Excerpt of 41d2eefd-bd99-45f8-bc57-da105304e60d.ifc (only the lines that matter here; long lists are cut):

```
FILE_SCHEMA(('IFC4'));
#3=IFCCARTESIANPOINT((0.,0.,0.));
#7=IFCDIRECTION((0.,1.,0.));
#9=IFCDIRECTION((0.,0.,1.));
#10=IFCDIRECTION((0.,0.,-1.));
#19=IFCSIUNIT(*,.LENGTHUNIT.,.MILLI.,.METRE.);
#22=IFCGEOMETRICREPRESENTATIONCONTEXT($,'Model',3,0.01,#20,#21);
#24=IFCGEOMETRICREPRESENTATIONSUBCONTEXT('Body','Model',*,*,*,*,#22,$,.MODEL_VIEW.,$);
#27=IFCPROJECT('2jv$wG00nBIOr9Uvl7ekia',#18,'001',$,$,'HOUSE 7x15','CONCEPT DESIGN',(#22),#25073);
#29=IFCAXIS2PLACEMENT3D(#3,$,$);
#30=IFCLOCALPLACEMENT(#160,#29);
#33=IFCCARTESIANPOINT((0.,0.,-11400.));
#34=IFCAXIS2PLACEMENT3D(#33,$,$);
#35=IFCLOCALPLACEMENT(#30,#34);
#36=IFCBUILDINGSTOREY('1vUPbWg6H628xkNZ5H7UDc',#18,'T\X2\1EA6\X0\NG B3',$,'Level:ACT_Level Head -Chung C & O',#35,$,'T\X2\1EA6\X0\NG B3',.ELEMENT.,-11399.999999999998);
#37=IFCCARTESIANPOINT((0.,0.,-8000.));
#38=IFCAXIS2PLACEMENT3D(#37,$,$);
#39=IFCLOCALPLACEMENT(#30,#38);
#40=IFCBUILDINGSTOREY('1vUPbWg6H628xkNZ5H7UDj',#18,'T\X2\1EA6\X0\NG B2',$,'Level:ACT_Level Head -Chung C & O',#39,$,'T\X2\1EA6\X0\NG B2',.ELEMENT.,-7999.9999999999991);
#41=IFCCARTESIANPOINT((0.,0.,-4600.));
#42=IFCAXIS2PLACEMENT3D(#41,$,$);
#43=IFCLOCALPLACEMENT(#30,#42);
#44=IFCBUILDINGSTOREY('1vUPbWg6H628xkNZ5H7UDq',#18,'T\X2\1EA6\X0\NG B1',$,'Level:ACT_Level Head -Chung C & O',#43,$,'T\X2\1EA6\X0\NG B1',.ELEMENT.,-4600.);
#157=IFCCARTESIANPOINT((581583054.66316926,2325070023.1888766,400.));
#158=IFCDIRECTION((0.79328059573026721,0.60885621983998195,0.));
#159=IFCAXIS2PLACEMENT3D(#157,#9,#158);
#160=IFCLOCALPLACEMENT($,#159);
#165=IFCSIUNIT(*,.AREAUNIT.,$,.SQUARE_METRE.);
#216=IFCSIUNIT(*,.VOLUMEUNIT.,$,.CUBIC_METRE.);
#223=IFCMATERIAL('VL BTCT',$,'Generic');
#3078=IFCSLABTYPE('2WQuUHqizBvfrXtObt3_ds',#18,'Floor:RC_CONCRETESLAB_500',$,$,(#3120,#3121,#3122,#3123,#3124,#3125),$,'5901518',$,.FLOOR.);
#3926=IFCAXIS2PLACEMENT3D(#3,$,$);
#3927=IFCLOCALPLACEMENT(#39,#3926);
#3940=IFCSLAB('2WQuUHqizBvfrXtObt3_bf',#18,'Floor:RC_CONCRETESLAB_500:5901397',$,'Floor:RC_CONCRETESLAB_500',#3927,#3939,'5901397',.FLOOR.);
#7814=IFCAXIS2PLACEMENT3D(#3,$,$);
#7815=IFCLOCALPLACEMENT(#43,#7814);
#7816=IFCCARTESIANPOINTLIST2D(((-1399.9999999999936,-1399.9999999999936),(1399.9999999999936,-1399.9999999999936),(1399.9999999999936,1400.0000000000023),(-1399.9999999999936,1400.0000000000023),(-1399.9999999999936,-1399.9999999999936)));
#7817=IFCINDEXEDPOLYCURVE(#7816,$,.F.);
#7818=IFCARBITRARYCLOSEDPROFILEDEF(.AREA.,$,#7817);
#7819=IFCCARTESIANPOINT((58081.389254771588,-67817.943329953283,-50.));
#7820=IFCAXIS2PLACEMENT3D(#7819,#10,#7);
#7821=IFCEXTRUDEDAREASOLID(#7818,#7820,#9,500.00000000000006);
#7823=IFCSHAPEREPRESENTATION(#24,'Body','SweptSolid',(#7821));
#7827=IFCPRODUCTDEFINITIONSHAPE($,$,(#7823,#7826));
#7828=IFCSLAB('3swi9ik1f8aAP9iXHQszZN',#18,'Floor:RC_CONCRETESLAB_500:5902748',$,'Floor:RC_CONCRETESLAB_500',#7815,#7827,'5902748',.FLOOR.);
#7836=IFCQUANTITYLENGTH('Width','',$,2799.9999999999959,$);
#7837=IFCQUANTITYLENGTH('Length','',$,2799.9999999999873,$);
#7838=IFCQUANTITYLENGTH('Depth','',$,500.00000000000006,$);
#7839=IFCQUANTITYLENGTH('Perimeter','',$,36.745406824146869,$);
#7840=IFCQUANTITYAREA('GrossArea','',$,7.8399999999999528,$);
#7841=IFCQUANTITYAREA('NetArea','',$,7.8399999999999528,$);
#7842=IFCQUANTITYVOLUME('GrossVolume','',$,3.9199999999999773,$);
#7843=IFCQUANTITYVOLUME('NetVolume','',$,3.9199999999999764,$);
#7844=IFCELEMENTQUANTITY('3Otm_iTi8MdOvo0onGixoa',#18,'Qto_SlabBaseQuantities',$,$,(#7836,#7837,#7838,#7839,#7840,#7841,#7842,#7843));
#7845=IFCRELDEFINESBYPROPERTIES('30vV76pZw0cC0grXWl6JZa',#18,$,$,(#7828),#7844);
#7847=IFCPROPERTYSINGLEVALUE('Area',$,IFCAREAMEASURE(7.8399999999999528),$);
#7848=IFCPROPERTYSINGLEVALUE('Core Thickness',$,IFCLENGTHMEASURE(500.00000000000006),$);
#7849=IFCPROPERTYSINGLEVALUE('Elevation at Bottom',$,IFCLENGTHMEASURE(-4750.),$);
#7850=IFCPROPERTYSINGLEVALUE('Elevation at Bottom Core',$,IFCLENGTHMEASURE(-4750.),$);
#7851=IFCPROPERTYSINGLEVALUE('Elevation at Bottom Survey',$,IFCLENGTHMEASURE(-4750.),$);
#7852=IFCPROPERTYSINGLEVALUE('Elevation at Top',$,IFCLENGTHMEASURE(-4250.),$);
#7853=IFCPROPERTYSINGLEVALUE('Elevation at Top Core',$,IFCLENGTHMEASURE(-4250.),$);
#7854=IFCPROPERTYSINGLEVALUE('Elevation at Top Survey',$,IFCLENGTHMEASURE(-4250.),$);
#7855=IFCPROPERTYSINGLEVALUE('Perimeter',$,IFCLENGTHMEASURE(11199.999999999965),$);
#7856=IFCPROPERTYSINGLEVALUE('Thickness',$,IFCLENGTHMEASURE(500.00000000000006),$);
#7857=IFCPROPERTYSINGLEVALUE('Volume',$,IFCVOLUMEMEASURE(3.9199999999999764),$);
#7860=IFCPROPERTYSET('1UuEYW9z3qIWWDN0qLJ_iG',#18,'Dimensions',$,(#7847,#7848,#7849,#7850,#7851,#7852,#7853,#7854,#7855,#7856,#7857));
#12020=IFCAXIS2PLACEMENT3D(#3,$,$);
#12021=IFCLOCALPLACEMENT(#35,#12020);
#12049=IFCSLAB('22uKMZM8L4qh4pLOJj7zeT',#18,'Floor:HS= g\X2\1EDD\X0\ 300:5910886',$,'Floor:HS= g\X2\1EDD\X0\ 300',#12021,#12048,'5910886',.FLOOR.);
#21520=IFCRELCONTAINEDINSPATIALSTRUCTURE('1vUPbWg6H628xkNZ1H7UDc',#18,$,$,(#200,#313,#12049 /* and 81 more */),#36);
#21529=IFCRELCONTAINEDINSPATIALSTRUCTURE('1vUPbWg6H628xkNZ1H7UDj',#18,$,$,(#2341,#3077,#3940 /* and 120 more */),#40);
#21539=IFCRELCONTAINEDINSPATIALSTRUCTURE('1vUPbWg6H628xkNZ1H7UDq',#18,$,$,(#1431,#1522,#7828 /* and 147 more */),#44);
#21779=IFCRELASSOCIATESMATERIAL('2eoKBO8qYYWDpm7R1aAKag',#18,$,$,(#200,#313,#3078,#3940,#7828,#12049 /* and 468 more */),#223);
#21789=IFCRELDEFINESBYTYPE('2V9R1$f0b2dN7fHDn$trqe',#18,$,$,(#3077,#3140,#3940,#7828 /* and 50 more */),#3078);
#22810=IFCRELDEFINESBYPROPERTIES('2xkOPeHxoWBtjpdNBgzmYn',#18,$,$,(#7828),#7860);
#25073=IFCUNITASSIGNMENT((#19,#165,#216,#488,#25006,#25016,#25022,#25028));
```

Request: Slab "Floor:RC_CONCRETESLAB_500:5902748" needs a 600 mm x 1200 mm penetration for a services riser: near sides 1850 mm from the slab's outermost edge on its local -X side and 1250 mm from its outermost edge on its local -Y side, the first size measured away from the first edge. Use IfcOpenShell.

```python
import numpy as np
import ifcopenshell
import ifcopenshell.api.feature
import ifcopenshell.api.geometry
import ifcopenshell.api.pset
import ifcopenshell.api.root
import ifcopenshell.geom
import ifcopenshell.util.element
import ifcopenshell.util.placement
import ifcopenshell.util.representation
import ifcopenshell.util.shape
import ifcopenshell.util.unit

model = ifcopenshell.open("41d2eefd-bd99-45f8-bc57-da105304e60d.ifc")
unit_scale = ifcopenshell.util.unit.calculate_unit_scale(model)
area_scale = ifcopenshell.util.unit.calculate_unit_scale(model, "AREAUNIT")
volume_scale = ifcopenshell.util.unit.calculate_unit_scale(model, "VOLUMEUNIT")
settings = ifcopenshell.geom.settings()


def volume(element):
    """Net volume in cubic metres, openings subtracted."""
    shape = ifcopenshell.geom.create_shape(settings, element)
    return ifcopenshell.util.shape.get_volume(shape.geometry)


slab = model.by_guid("3swi9ik1f8aAP9iXHQszZN")
before = volume(slab)

# Extent in the slab's own axes, in metres. The edges named are its -X and -Y sides.
slab_shape = ifcopenshell.geom.create_shape(settings, slab)
vertices = ifcopenshell.util.shape.get_vertices(slab_shape.geometry)
x_min, y_min, bottom = vertices.min(axis=0)
top = vertices[:, 2].max()

opening = ifcopenshell.api.root.create_entity(model, ifc_class="IfcOpeningElement", name="Services riser opening", predefined_type="OPENING")
context = ifcopenshell.util.representation.get_context(model, "Model", "Body", "MODEL_VIEW")
width, depth = 0.6, 1.2
outline = [(0.0, 0.0), (width, 0.0), (width, depth), (0.0, depth), (0.0, 0.0)]
# Overshoot both faces by 50 mm so the cut is clean.
shape = ifcopenshell.api.geometry.add_slab_representation(
    model, context=context, depth=top - bottom + 0.1, polyline=outline
)
ifcopenshell.api.geometry.assign_representation(model, product=opening, representation=shape)

matrix = ifcopenshell.util.placement.get_local_placement(slab.ObjectPlacement)
matrix[:, 3] = matrix @ np.append(np.array([x_min + 1.85, y_min + 1.25, bottom - 0.05]) / unit_scale, 1.0)
ifcopenshell.api.geometry.edit_object_placement(model, product=opening, matrix=matrix, is_si=False)
ifcopenshell.api.feature.add_feature(model, feature=opening, element=slab)

after = volume(slab)

# Update the slab's stored quantities.
qto = model.by_id(ifcopenshell.util.element.get_pset(slab, "Qto_SlabBaseQuantities", should_inherit=False)["id"])
ifcopenshell.api.pset.edit_qto(model, qto=qto, properties={
    "NetArea": after / (top - bottom) / area_scale,
    "NetVolume": after / volume_scale,
})
pset = model.by_id(ifcopenshell.util.element.get_pset(slab, "Dimensions", should_inherit=False)["id"])
ifcopenshell.api.pset.edit_pset(model, pset=pset, properties={
    "Area": model.create_entity("IfcAreaMeasure", after / (top - bottom) / area_scale),
    "Volume": model.create_entity("IfcVolumeMeasure", after / volume_scale),
})

print(f"slab volume {before:.3f} -> {after:.3f} m3")

model.write("41d2eefd-bd99-45f8-bc57-da105304e60d_edited.ifc")
```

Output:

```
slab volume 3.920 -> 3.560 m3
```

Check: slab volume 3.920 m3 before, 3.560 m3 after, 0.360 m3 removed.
